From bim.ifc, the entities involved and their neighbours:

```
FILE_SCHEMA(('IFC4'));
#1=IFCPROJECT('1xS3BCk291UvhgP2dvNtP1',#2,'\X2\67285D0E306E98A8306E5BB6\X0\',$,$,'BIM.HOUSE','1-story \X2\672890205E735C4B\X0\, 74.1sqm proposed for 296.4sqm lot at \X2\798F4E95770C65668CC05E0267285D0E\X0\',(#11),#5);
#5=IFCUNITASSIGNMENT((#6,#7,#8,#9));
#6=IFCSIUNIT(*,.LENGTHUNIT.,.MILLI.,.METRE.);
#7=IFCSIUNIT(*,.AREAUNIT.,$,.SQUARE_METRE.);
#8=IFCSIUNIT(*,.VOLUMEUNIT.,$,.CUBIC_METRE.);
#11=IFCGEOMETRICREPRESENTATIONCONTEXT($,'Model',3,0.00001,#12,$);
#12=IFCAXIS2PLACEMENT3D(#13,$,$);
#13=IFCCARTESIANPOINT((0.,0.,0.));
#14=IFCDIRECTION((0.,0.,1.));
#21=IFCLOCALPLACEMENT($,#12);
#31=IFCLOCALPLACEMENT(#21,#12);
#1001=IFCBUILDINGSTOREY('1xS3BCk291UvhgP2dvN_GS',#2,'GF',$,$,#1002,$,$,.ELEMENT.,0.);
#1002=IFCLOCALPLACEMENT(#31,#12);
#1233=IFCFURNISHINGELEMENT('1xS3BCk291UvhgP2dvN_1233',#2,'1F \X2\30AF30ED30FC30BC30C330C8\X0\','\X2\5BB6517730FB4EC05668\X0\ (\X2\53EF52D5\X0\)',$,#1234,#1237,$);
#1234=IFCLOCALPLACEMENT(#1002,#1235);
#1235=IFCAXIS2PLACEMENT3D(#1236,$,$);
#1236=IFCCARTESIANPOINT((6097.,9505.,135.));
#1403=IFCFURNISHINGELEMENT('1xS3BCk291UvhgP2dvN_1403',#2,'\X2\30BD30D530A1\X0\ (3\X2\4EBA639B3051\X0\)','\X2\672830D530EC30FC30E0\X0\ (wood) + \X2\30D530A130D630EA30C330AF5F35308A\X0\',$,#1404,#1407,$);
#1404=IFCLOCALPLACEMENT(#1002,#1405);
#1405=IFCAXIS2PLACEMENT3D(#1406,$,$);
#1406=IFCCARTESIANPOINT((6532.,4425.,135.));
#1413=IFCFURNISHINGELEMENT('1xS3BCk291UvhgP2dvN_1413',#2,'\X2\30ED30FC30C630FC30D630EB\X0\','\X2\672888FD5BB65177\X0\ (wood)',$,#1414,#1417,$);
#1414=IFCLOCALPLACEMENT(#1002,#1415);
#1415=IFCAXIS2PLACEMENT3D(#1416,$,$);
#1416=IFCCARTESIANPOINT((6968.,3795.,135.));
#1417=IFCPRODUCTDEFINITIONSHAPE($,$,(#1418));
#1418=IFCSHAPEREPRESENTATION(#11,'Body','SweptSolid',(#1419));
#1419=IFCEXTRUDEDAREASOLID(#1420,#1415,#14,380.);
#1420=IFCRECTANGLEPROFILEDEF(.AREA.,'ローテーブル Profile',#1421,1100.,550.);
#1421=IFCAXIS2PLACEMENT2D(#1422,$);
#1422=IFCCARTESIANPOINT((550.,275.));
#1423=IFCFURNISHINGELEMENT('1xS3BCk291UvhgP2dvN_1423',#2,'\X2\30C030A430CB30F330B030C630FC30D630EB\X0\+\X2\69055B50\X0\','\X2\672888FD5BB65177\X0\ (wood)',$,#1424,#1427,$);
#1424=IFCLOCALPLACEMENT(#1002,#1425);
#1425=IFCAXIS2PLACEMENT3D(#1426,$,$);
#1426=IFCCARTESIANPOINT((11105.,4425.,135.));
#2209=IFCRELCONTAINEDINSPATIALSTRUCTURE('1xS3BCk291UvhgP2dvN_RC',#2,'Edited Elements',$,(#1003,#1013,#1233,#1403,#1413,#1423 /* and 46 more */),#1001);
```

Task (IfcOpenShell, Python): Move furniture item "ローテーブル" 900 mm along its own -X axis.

```python
import ifcopenshell
import ifcopenshell.api.geometry
import ifcopenshell.util.placement

model = ifcopenshell.open("bim.ifc")

item = model.by_guid("1xS3BCk291UvhgP2dvN_1413")
matrix = ifcopenshell.util.placement.get_local_placement(item.ObjectPlacement)
matrix[:3, 3] -= matrix[:3, 0] * 900.0
ifcopenshell.api.geometry.edit_object_placement(model, product=item, matrix=matrix, is_si=False)

print(ifcopenshell.util.placement.get_local_placement(item.ObjectPlacement).round(3) + 0.0)

model.write("bim-out.ifc")
```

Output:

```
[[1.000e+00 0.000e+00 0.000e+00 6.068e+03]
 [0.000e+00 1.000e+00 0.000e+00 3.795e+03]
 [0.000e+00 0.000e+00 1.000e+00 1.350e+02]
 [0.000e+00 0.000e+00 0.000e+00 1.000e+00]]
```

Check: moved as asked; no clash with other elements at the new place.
